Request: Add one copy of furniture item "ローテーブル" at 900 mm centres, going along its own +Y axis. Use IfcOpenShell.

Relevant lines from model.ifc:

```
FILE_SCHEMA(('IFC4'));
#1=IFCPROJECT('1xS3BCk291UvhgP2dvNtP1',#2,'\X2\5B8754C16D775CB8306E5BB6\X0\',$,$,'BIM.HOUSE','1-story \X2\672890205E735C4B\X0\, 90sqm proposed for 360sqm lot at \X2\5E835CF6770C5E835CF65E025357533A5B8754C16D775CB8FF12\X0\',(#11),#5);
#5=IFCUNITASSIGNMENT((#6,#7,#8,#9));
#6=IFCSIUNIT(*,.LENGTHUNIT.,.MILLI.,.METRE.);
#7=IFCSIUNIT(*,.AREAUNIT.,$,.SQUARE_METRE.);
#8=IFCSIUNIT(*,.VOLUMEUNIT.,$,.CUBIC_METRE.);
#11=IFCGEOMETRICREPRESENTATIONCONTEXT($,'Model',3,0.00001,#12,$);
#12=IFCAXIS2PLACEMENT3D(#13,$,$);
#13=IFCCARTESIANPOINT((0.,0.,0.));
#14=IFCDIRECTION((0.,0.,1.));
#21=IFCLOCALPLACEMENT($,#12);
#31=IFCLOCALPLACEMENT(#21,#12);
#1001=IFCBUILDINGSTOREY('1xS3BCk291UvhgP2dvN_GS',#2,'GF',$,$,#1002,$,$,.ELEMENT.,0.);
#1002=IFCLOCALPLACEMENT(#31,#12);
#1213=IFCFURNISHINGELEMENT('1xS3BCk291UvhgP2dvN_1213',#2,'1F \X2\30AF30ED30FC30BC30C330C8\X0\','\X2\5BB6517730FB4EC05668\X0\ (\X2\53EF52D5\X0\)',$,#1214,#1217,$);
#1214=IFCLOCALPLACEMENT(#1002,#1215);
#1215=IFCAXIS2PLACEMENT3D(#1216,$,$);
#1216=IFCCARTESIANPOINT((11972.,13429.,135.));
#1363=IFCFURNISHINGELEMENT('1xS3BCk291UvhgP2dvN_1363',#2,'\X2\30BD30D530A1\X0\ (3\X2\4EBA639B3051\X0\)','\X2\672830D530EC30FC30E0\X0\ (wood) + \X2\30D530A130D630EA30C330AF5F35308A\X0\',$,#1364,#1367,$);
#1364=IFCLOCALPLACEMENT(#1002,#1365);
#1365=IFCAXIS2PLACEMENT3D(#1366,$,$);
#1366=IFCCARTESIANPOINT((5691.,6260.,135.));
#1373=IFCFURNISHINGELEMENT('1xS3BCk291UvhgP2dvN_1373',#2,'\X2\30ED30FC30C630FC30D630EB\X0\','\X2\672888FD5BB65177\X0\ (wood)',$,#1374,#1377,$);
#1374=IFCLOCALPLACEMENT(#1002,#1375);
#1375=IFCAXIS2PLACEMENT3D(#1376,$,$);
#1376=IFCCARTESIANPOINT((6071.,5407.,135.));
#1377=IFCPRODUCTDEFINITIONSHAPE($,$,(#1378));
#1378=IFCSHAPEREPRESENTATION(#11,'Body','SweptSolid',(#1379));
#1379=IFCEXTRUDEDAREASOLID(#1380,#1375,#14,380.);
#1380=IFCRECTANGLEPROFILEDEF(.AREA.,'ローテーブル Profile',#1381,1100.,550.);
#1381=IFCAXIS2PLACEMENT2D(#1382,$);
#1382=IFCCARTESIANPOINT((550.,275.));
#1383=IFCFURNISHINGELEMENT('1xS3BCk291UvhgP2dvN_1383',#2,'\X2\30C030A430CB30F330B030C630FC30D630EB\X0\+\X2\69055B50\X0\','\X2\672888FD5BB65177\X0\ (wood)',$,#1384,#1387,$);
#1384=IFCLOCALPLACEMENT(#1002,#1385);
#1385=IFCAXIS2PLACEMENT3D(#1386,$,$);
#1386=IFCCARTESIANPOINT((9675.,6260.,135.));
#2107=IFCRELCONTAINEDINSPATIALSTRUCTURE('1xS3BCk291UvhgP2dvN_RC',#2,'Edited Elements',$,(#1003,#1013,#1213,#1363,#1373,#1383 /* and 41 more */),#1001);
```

```python
import ifcopenshell
import ifcopenshell.api.geometry
import ifcopenshell.api.root
import ifcopenshell.util.element
import ifcopenshell.util.placement
import ifcopenshell.util.unit

model = ifcopenshell.open("model.ifc")
unit_scale = ifcopenshell.util.unit.calculate_unit_scale(model)


def reuse_history(source, copy):
    """copy_class also copies each property set's owner history, people and application; keep the originals."""
    for rel in copy.IsDefinedBy:
        if rel.is_a("IfcRelDefinesByProperties") and (history := rel.RelatingPropertyDefinition.OwnerHistory):
            rel.RelatingPropertyDefinition.OwnerHistory = source.OwnerHistory
            ifcopenshell.util.element.remove_deep2(model, history)


source = model.by_id(1373)
base = ifcopenshell.util.placement.get_local_placement(source.ObjectPlacement)
step = base[:3, 1] * 0.9 / unit_scale

for i in range(1, 2):
    copy = ifcopenshell.api.root.copy_class(model, product=source)
    copy.Representation = ifcopenshell.util.element.copy_deep(
        model, source.Representation, exclude=["IfcGeometricRepresentationContext", "IfcRepresentationMap"]
    )
    reuse_history(source, copy)
    matrix = base.copy()
    matrix[:3, 3] += i * step
    print("added at", matrix[:3, 3].round(3) + 0.0)
    ifcopenshell.api.geometry.edit_object_placement(model, product=copy, matrix=matrix, is_si=False)

model.write("model_updated.ifc")
```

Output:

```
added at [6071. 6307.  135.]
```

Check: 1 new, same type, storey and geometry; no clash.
